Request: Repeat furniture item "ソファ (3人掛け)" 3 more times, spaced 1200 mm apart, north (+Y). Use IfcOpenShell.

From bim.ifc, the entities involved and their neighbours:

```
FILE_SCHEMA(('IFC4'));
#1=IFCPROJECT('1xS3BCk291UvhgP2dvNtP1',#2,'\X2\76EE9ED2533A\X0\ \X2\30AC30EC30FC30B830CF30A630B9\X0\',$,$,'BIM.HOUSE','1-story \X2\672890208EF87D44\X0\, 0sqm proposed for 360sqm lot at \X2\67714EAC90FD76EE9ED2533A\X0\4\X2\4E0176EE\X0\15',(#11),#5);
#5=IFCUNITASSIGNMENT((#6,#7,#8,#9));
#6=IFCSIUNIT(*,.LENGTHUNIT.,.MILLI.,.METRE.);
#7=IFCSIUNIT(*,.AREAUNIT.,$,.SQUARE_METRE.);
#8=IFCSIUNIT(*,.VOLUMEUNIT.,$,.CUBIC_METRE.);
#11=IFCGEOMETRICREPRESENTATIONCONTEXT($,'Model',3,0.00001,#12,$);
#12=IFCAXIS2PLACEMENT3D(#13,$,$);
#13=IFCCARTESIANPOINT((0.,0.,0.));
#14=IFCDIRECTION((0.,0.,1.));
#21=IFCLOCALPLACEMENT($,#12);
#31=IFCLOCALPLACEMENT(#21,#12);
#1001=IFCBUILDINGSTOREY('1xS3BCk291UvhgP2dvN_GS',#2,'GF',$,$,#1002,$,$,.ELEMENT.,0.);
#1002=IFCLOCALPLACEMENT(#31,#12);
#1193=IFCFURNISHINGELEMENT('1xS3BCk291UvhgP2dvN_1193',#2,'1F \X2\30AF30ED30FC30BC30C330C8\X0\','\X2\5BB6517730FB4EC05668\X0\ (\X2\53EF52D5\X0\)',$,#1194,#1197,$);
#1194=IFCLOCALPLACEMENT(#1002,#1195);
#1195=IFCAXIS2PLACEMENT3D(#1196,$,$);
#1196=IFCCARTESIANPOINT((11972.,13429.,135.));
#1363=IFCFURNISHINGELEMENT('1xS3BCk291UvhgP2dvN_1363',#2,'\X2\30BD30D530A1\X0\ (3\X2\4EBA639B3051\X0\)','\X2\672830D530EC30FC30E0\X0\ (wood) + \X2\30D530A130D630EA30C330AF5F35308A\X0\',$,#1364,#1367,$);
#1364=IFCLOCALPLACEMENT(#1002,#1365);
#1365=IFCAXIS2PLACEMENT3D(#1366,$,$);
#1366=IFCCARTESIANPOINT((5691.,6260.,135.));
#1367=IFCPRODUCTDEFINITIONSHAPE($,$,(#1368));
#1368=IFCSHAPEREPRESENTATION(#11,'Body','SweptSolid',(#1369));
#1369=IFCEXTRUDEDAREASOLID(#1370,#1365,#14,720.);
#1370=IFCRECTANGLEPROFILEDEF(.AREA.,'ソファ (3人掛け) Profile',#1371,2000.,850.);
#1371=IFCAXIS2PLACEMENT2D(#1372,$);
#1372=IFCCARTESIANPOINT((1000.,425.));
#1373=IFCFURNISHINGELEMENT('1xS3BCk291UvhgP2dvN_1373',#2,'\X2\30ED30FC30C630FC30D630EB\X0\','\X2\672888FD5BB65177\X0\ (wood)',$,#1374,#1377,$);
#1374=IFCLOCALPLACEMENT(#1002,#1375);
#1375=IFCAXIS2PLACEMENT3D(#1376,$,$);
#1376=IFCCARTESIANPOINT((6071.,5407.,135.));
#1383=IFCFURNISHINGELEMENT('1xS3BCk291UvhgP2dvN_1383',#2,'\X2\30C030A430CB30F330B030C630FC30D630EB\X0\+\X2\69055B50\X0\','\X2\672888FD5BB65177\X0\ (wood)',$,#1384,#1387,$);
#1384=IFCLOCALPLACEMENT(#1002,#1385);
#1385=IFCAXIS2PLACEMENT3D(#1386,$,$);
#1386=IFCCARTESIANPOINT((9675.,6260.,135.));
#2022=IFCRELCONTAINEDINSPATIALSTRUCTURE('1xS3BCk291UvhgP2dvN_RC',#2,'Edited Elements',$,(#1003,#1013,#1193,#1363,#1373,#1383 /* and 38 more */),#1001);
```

```python
import numpy as np
import ifcopenshell
import ifcopenshell.api.geometry
import ifcopenshell.api.root
import ifcopenshell.util.element
import ifcopenshell.util.placement
import ifcopenshell.util.unit

model = ifcopenshell.open("bim.ifc")
unit_scale = ifcopenshell.util.unit.calculate_unit_scale(model)


def reuse_history(source, copy):
    """copy_class also copies each property set's owner history, people and application; keep the originals."""
    for rel in copy.IsDefinedBy:
        if rel.is_a("IfcRelDefinesByProperties") and (history := rel.RelatingPropertyDefinition.OwnerHistory):
            rel.RelatingPropertyDefinition.OwnerHistory = source.OwnerHistory
            ifcopenshell.util.element.remove_deep2(model, history)


source = model.by_id(1363)
base = ifcopenshell.util.placement.get_local_placement(source.ObjectPlacement)
step = np.array([0.0, 1.0, 0.0]) * 1.2 / unit_scale

for i in range(1, 4):
    copy = ifcopenshell.api.root.copy_class(model, product=source)
    copy.Representation = ifcopenshell.util.element.copy_deep(
        model, source.Representation, exclude=["IfcGeometricRepresentationContext", "IfcRepresentationMap"]
    )
    reuse_history(source, copy)
    matrix = base.copy()
    matrix[:3, 3] += i * step
    print("added at", matrix[:3, 3].round(3) + 0.0)
    ifcopenshell.api.geometry.edit_object_placement(model, product=copy, matrix=matrix, is_si=False)

model.write("bim_edited.ifc")
```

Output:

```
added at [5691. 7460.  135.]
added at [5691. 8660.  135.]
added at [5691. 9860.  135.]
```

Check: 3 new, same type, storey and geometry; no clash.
